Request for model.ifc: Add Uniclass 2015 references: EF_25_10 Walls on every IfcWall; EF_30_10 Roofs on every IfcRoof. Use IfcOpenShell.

First a look at what the model holds.

```python
import ifcopenshell

model = ifcopenshell.open("model.ifc")
print(model.schema)
print("classifications:", [c.Name for c in model.by_type("IfcClassification")])
for ifc_class in ("IfcDoor", "IfcRoof", "IfcStair", "IfcWall", "IfcWindow"):
    print(ifc_class, len(model.by_type(ifc_class)))
```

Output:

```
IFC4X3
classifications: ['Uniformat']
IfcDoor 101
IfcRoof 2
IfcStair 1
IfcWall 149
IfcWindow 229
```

```python
import ifcopenshell
import ifcopenshell.api.classification

model = ifcopenshell.open("model.ifc")

system = ifcopenshell.api.classification.add_classification(model, classification="Uniclass 2015")

codes = {
    "IfcWall": ("EF_25_10", "Walls"),
    "IfcRoof": ("EF_30_10", "Roofs"),
}
for ifc_class, (code, name) in codes.items():
    products = model.by_type(ifc_class)
    ifcopenshell.api.classification.add_reference(
        model, products=products, classification=system, identification=code, name=name
    )
    print(code, len(products))

model.write("model_rev.ifc")
```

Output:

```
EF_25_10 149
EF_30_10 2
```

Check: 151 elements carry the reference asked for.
